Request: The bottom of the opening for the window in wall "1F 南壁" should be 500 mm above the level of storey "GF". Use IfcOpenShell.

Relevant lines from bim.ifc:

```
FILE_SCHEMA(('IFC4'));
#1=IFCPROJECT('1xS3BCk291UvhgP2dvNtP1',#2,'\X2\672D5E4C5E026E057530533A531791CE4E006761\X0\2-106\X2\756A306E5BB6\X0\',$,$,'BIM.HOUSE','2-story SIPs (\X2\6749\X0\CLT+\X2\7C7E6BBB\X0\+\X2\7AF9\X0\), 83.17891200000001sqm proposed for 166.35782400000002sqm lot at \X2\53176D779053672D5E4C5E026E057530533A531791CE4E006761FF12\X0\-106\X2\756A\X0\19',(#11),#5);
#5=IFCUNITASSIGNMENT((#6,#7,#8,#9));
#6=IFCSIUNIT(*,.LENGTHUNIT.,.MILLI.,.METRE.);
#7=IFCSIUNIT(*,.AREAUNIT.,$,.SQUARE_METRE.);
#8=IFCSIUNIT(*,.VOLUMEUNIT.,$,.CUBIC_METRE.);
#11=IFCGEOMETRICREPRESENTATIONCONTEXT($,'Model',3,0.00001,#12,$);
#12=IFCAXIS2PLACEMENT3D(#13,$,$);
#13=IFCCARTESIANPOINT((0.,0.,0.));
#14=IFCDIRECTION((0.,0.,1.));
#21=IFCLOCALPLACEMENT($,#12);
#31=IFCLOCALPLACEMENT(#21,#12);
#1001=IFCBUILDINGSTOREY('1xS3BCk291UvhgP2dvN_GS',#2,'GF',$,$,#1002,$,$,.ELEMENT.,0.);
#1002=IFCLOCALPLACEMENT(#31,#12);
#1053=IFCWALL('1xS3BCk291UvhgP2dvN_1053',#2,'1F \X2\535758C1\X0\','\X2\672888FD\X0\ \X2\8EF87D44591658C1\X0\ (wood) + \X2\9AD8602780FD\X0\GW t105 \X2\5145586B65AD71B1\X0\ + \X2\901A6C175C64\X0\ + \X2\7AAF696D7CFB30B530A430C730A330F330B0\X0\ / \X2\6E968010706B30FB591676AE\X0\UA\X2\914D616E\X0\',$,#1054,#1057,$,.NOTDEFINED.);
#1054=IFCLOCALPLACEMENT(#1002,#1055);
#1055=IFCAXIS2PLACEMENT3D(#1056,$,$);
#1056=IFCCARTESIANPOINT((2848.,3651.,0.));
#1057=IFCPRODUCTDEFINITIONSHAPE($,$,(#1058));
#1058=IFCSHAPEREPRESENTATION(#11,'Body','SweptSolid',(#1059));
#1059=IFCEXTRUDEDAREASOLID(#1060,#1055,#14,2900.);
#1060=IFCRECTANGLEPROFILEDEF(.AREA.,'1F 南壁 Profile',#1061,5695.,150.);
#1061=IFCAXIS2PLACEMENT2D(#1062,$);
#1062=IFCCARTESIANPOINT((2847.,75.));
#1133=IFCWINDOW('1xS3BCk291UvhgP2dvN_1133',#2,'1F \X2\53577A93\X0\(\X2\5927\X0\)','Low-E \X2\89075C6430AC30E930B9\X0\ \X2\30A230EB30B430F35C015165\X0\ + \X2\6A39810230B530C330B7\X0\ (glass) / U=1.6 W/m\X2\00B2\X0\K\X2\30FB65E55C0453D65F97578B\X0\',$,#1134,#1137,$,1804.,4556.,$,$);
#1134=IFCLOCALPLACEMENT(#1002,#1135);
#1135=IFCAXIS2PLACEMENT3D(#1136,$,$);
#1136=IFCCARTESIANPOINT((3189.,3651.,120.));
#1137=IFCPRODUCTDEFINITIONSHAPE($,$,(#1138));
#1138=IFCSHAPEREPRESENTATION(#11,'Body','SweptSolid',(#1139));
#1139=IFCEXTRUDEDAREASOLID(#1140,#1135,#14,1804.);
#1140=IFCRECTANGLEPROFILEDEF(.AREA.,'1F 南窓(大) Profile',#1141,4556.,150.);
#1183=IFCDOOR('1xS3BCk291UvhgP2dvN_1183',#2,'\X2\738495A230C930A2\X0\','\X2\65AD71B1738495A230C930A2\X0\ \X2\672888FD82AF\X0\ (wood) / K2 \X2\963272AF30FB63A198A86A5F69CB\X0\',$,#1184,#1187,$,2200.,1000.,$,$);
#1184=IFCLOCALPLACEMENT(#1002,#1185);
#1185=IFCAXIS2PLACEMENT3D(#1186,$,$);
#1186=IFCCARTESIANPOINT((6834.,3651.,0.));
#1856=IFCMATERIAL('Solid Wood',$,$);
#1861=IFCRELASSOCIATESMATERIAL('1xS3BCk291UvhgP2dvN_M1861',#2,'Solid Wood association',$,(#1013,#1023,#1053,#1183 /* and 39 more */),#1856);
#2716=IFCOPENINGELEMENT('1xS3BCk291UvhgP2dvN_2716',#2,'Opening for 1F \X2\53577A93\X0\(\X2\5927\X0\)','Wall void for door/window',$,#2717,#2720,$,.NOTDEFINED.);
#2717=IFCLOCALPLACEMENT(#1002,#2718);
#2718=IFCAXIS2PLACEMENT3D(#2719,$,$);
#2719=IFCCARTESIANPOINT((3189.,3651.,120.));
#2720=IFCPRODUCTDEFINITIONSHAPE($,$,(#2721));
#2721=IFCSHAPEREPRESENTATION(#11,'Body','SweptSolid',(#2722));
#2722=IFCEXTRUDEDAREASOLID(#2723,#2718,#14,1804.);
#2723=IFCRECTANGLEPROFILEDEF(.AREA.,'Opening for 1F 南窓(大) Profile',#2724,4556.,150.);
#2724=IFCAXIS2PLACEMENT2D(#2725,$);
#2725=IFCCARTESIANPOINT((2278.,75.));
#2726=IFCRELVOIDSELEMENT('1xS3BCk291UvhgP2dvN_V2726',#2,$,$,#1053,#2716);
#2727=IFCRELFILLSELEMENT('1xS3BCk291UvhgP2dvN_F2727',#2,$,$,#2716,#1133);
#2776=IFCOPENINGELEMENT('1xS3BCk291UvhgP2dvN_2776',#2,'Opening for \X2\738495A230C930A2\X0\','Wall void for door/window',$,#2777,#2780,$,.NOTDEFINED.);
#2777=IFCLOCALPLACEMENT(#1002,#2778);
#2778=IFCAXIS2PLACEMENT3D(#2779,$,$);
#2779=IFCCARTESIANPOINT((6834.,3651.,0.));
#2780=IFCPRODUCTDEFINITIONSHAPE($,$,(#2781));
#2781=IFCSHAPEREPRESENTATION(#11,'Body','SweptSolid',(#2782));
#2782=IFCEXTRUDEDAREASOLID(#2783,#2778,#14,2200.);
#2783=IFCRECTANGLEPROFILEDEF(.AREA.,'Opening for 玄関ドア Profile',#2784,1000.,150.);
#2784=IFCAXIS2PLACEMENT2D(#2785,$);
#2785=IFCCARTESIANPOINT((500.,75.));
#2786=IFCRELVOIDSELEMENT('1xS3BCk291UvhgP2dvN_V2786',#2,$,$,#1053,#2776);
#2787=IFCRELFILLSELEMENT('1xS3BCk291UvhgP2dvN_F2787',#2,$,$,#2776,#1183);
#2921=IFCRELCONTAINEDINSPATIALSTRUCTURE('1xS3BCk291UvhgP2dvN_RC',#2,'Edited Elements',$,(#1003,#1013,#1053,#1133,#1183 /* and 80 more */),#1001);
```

```python
import numpy as np
import ifcopenshell
import ifcopenshell.api.geometry
import ifcopenshell.geom
import ifcopenshell.util.element
import ifcopenshell.util.placement
import ifcopenshell.util.shape
import ifcopenshell.util.unit

model = ifcopenshell.open("bim.ifc")
unit_scale = ifcopenshell.util.unit.calculate_unit_scale(model)

window = model.by_guid("1xS3BCk291UvhgP2dvN_1133")
opening = window.FillsVoids[0].RelatingOpeningElement
storey = ifcopenshell.util.element.get_container(window, ifc_class="IfcBuildingStorey")
level = ifcopenshell.util.placement.get_local_placement(storey.ObjectPlacement)[2, 3]

# The opening's origin need not be at the sill, so measure its lowest point.
shape = ifcopenshell.geom.create_shape(ifcopenshell.geom.settings(), opening)
bottom = ifcopenshell.util.shape.get_shape_bottom_elevation(shape, shape.geometry) / unit_scale
dz = level + 500.0 - bottom

shift = np.array([0.0, 0.0, dz])
# The window is not placed relative to its opening, so move both.
for product in (opening, window):
    matrix = ifcopenshell.util.placement.get_local_placement(product.ObjectPlacement)
    matrix[:3, 3] += shift
    ifcopenshell.api.geometry.edit_object_placement(model, product=product, matrix=matrix, is_si=False)

print(f"moved by {dz * unit_scale:+.3f} m")

model.write("bim_edited.ifc")
```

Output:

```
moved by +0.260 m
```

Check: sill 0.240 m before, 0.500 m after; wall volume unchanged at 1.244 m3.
